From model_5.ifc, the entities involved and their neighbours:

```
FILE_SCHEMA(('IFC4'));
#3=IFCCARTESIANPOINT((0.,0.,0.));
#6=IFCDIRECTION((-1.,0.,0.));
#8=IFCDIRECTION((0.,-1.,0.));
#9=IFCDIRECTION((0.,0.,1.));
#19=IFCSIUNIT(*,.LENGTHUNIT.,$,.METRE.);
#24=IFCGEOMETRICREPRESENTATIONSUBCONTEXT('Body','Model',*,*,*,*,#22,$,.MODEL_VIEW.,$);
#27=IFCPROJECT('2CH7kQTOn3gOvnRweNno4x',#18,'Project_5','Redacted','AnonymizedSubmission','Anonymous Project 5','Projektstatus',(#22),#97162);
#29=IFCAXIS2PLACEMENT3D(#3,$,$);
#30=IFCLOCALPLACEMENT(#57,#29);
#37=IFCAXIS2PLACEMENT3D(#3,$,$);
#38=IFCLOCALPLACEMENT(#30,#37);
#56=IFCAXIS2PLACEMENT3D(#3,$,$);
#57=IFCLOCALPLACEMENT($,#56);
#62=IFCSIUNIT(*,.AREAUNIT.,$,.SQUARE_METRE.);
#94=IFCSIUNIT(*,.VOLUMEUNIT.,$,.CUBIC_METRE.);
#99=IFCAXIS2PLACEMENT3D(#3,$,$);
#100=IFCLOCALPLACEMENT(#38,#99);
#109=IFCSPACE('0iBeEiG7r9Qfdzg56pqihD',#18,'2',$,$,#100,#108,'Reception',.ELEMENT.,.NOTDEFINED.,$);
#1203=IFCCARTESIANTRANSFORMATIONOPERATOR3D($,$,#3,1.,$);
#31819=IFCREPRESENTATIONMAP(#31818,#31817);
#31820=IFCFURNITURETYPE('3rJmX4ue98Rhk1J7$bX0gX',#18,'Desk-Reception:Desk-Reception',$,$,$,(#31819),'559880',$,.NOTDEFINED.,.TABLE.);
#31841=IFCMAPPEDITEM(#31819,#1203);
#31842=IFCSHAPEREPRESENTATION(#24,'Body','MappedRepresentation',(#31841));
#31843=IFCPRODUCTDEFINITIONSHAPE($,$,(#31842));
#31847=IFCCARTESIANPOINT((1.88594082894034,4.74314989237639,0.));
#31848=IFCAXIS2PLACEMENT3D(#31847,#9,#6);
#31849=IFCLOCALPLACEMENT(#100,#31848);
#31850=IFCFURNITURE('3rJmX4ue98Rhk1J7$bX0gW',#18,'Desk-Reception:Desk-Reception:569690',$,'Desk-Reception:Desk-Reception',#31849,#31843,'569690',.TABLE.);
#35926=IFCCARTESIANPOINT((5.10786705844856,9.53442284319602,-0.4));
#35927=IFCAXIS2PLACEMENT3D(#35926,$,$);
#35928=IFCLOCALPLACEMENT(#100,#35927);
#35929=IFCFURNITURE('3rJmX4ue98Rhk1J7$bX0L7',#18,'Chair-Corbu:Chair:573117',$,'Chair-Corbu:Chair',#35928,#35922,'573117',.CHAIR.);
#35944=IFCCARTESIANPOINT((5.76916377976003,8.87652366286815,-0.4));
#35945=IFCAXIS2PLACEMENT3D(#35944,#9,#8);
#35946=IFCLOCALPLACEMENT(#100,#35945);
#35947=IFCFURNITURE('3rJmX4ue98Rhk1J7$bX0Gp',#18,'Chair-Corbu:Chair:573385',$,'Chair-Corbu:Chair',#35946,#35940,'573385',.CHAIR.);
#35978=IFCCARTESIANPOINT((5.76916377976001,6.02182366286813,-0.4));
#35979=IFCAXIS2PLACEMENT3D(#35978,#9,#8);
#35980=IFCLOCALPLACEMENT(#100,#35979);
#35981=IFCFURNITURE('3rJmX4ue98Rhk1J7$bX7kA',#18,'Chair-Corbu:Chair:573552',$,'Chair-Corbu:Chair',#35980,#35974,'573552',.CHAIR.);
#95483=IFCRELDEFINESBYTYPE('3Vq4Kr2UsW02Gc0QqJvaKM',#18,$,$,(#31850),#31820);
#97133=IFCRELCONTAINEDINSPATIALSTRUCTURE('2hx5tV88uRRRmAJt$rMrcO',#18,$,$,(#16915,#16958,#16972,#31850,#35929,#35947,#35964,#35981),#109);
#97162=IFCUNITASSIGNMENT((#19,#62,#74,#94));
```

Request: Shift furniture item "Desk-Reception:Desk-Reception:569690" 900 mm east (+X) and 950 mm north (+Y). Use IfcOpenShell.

```python
import ifcopenshell
import ifcopenshell.api.geometry
import ifcopenshell.util.placement

model = ifcopenshell.open("model_5.ifc")

item = model.by_guid("3rJmX4ue98Rhk1J7$bX0gW")
matrix = ifcopenshell.util.placement.get_local_placement(item.ObjectPlacement)
matrix[0, 3] += 0.9
matrix[1, 3] += 0.95
ifcopenshell.api.geometry.edit_object_placement(model, product=item, matrix=matrix, is_si=False)

print(ifcopenshell.util.placement.get_local_placement(item.ObjectPlacement).round(3) + 0.0)

model.write("model_5_edited.ifc")
```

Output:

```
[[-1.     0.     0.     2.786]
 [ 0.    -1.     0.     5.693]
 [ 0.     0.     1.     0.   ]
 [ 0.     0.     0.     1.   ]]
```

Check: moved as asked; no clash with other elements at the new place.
